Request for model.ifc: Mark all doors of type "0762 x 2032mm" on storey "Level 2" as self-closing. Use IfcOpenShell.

First a look at what the model holds.

```python
import ifcopenshell
import ifcopenshell.util.element

model = ifcopenshell.open("model.ifc")
print(model.schema)
storey = next(s for s in model.by_type("IfcBuildingStorey") if s.Name == "Level 2")
doors = [e for e in ifcopenshell.util.element.get_decomposition(storey) if e.is_a("IfcDoor")]
seen = {}
for e in doors:
    element_type = ifcopenshell.util.element.get_type(e)
    key = (element_type.Name if element_type != e and element_type else None, ifcopenshell.util.element.get_pset(e, "Pset_DoorCommon", "SelfClosing"))
    seen[key] = seen.get(key, 0) + 1
for (name, value), count in sorted(seen.items(), key=str):
    print(count, "x", name, "|", value)
```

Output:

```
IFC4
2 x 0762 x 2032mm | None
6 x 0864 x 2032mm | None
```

```python
import ifcopenshell
import ifcopenshell.api.pset
import ifcopenshell.util.element

model = ifcopenshell.open("model.ifc")

storey = next(s for s in model.by_type("IfcBuildingStorey") if s.Name == "Level 2")
doors = [e for e in ifcopenshell.util.element.get_decomposition(storey) if e.is_a("IfcDoor")]

count = 0
for e in doors:
    element_type = ifcopenshell.util.element.get_type(e)
    if element_type in (None, e) or element_type.Name != "0762 x 2032mm":
        continue
    # add_pset returns the element's existing set when there is one.
    pset = ifcopenshell.api.pset.add_pset(model, product=e, name="Pset_DoorCommon")
    ifcopenshell.api.pset.edit_pset(model, pset=pset, properties={"SelfClosing": True})
    count += 1

print(count, "doors updated")

model.write("model_updated.ifc")
```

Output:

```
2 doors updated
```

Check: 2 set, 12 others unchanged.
